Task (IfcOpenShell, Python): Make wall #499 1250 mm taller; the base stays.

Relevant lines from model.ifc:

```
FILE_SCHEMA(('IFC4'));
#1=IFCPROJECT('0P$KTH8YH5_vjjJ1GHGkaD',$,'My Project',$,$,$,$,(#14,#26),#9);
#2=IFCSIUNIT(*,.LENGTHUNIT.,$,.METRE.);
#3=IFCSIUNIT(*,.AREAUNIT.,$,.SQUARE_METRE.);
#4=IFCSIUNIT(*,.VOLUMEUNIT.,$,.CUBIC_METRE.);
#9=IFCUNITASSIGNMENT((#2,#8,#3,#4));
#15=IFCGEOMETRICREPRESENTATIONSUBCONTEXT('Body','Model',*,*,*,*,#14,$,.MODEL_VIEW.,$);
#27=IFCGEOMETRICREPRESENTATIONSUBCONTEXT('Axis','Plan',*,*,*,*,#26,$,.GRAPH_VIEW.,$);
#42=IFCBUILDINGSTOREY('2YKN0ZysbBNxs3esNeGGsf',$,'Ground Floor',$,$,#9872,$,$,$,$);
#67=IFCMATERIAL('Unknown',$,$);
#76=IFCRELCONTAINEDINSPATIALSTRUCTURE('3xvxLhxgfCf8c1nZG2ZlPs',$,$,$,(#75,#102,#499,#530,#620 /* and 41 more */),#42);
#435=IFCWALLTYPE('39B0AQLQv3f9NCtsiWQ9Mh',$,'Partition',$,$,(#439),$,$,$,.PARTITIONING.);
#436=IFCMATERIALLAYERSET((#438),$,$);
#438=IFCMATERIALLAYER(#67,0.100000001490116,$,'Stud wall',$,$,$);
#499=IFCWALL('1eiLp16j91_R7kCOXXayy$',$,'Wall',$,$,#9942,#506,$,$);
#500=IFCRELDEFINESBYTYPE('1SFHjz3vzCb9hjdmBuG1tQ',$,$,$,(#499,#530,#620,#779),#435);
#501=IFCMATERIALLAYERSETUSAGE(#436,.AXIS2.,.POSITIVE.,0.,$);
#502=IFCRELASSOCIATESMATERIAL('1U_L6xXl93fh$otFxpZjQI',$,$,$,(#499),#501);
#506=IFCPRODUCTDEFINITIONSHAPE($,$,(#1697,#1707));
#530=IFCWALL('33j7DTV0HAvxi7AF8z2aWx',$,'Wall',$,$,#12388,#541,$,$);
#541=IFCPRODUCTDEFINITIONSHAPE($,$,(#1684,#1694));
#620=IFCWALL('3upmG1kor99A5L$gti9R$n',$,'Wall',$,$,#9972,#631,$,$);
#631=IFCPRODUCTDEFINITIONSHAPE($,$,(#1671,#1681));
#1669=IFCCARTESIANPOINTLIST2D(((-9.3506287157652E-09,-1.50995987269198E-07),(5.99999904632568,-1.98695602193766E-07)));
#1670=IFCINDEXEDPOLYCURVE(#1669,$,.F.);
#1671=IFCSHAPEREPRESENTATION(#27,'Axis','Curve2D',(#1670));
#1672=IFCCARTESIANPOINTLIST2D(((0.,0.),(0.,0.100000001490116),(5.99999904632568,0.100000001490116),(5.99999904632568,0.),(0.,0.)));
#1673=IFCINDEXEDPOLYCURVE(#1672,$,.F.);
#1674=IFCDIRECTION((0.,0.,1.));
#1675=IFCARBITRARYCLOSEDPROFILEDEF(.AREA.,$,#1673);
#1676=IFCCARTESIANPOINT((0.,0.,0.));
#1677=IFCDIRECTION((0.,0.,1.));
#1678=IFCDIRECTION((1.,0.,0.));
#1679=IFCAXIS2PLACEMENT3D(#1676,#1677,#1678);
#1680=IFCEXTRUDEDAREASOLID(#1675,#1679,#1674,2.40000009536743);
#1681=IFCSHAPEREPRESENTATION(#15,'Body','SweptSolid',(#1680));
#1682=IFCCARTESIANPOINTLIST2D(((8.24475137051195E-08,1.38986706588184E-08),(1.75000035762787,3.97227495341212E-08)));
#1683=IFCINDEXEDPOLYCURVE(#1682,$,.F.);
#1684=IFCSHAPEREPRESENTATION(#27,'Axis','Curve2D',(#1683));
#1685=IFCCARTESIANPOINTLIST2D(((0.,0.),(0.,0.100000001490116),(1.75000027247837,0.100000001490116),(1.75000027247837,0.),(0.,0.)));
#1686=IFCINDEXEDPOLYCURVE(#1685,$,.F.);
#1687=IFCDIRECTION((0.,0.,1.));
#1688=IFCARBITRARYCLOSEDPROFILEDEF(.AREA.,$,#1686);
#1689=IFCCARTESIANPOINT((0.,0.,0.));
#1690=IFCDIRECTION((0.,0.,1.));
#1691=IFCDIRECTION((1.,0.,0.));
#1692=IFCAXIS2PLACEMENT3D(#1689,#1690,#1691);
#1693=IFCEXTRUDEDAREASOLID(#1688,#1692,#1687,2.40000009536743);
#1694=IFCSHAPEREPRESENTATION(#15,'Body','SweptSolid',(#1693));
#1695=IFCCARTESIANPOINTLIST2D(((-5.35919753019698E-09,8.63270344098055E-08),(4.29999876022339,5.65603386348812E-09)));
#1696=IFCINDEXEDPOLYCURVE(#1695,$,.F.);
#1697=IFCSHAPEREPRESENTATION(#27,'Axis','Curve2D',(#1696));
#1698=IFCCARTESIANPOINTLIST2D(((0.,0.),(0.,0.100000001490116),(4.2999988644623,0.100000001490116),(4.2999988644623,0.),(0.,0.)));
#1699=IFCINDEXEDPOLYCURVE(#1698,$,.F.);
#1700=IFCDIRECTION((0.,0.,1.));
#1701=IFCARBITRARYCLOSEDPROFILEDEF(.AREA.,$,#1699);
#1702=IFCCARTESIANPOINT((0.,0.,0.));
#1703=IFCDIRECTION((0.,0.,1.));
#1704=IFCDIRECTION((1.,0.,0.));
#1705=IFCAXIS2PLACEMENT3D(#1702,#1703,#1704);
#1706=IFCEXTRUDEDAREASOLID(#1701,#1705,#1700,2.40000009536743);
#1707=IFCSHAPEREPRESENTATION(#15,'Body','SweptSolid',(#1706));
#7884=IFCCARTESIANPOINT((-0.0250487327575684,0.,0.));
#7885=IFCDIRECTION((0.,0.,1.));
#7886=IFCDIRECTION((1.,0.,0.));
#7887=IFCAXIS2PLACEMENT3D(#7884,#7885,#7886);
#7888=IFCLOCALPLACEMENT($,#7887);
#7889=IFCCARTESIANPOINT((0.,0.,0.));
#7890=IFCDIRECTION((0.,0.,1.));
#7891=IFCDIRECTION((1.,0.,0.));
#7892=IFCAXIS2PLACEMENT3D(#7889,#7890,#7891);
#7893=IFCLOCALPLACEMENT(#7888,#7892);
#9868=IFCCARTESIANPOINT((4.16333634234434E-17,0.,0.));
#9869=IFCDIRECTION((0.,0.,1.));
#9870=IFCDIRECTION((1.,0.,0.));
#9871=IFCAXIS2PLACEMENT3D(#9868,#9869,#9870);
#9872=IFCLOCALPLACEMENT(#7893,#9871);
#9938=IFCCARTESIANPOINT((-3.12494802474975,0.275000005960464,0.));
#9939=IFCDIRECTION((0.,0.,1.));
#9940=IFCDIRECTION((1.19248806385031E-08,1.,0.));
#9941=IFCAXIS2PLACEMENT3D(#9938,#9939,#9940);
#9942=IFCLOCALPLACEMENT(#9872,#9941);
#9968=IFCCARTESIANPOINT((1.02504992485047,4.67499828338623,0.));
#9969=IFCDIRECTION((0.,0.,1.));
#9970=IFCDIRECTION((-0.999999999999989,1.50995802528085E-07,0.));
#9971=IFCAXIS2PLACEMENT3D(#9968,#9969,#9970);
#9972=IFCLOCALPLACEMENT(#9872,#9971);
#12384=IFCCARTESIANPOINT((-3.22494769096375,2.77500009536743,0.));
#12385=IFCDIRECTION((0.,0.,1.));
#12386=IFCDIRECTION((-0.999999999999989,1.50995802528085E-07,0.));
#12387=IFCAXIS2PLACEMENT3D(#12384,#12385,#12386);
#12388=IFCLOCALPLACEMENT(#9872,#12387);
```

```python
import ifcopenshell
import ifcopenshell.geom
import ifcopenshell.util.representation
import ifcopenshell.util.shape

model = ifcopenshell.open("model.ifc")
settings = ifcopenshell.geom.settings()


def volume(element):
    """Net volume in cubic metres, openings subtracted."""
    shape = ifcopenshell.geom.create_shape(settings, element)
    return ifcopenshell.util.shape.get_volume(shape.geometry)


wall = model.by_guid("1eiLp16j91_R7kCOXXayy$")
before = volume(wall)

body = ifcopenshell.util.representation.get_representation(wall, "Model", "Body")
solid = body.Items[0]
old_height = solid.Depth
solid.Depth += 1.25
after = volume(wall)

print(f"height {old_height:g} -> {solid.Depth:g}, volume {before:.3f} -> {after:.3f} m3")

model.write("model_updated.ifc")
```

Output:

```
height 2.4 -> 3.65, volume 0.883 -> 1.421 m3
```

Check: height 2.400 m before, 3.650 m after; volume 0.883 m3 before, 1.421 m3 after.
